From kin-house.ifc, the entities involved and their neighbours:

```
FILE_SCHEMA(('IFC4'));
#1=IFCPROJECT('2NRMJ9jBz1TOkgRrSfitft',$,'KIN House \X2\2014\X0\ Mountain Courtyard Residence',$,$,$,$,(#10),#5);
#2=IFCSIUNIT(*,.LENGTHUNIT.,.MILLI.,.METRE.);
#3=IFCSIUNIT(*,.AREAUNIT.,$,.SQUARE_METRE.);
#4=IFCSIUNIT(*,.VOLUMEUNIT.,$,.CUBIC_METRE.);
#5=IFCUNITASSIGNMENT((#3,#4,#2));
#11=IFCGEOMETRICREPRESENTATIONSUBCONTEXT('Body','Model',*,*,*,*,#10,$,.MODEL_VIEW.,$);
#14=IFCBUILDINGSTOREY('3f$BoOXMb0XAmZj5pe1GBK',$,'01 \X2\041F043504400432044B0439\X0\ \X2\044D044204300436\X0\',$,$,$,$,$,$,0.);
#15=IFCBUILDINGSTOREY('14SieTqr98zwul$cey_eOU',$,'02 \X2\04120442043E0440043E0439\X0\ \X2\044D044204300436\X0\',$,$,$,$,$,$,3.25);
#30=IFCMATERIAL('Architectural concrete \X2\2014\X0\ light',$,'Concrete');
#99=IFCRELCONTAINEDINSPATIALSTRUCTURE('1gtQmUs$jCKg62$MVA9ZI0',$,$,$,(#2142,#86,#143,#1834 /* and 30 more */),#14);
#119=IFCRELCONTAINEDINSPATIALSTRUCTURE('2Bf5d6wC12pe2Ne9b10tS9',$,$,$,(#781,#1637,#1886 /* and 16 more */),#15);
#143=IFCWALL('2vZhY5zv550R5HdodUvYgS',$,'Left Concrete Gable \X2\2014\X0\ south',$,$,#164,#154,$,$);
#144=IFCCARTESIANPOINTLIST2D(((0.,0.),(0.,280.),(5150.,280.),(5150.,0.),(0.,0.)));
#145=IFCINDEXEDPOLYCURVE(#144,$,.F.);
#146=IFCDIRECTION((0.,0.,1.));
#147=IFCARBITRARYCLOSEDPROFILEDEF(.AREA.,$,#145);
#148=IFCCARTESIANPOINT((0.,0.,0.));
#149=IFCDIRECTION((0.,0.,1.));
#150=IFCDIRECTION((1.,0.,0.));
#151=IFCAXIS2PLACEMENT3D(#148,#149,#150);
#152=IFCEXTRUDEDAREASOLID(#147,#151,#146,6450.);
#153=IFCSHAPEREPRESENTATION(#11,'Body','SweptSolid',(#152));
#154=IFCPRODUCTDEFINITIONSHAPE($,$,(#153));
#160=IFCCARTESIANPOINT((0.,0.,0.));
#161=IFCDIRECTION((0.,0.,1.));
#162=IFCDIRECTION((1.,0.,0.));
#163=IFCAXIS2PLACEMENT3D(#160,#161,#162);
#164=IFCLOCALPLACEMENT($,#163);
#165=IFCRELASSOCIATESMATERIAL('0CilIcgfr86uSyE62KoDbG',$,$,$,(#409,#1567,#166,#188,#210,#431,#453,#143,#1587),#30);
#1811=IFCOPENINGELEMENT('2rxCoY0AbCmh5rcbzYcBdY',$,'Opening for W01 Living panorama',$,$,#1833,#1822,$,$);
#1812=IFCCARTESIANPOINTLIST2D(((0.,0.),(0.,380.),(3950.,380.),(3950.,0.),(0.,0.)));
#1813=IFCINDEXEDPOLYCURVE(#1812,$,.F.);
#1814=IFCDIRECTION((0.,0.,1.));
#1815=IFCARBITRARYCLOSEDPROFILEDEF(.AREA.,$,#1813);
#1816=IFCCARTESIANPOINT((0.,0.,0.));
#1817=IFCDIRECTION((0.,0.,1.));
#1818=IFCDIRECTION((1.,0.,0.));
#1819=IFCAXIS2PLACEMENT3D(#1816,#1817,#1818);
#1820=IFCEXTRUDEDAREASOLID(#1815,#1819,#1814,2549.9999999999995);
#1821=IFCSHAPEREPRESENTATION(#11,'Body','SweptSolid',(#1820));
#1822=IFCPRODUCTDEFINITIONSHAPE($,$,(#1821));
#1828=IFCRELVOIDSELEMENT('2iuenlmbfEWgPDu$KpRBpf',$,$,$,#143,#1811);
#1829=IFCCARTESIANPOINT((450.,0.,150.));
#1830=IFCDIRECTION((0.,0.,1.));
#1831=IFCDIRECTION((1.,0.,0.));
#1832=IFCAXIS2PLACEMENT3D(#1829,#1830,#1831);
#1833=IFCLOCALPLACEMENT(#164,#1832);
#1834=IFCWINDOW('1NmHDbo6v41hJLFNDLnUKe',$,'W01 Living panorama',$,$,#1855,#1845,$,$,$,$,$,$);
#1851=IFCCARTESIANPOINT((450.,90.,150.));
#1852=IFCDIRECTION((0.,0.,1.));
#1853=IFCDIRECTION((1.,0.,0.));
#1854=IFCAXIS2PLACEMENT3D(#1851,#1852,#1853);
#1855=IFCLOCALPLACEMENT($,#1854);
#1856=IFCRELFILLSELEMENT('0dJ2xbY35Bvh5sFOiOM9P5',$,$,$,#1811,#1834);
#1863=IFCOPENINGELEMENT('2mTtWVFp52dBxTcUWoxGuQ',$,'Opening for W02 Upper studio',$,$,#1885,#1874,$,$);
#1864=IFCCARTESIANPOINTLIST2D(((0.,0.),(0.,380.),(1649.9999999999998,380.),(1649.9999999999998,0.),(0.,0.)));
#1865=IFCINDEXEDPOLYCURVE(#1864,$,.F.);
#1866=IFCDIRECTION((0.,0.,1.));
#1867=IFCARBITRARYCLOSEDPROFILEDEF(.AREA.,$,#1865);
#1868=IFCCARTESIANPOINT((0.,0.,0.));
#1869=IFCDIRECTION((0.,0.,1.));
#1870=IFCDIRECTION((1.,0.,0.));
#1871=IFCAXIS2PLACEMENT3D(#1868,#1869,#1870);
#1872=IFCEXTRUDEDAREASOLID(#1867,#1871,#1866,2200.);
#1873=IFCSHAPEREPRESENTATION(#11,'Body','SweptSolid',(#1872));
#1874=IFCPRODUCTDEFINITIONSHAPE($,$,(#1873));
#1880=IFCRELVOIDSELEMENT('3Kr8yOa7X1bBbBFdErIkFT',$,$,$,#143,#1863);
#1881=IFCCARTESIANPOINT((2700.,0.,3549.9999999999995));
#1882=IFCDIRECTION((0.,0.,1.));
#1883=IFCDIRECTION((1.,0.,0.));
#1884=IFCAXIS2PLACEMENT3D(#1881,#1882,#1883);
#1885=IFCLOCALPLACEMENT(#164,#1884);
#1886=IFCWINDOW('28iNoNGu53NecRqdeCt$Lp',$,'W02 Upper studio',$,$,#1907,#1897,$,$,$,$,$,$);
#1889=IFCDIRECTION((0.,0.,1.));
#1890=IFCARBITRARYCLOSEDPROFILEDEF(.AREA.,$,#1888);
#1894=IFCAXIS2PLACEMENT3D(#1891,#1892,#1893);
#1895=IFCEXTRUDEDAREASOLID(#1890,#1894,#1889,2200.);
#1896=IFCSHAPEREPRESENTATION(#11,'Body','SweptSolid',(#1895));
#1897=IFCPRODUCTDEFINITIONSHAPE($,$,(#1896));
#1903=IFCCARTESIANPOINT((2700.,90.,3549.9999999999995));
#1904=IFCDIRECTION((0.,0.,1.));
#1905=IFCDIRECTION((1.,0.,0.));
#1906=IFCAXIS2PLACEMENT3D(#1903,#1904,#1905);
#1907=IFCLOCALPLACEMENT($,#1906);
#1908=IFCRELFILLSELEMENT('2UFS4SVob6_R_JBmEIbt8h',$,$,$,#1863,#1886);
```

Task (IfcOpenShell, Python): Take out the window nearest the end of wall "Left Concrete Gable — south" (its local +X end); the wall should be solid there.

```python
import ifcopenshell
import ifcopenshell.api.feature
import ifcopenshell.api.root
import ifcopenshell.geom
import ifcopenshell.util.shape

model = ifcopenshell.open("kin-house.ifc")
settings = ifcopenshell.geom.settings()


def volume(element):
    """Net volume in cubic metres, openings subtracted."""
    shape = ifcopenshell.geom.create_shape(settings, element)
    return ifcopenshell.util.shape.get_volume(shape.geometry)


window = model.by_guid("28iNoNGu53NecRqdeCt$Lp")
opening = window.FillsVoids[0].RelatingOpeningElement
wall = opening.VoidsElements[0].RelatingBuildingElement
before = volume(wall)

ifcopenshell.api.root.remove_product(model, product=window)
ifcopenshell.api.feature.remove_feature(model, feature=opening)

after = volume(wall)

print(f"wall volume {before:.3f} -> {after:.3f} m3")

model.write("kin-house_v2.ifc")
```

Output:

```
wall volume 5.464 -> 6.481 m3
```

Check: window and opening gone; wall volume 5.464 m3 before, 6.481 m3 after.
